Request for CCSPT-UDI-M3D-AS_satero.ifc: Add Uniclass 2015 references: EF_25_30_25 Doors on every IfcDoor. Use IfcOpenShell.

First a look at what the model holds.

```python
import ifcopenshell

model = ifcopenshell.open("CCSPT-UDI-M3D-AS_satero.ifc")
print(model.schema)
print("classifications:", [c.Name for c in model.by_type("IfcClassification")])
for ifc_class in ("IfcDoor", "IfcRoof", "IfcStair", "IfcWall", "IfcWindow"):
    print(ifc_class, len(model.by_type(ifc_class)))
```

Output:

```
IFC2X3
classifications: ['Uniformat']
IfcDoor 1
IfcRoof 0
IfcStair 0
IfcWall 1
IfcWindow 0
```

```python
import ifcopenshell
import ifcopenshell.api.classification

model = ifcopenshell.open("CCSPT-UDI-M3D-AS_satero.ifc")

# IFC2X3 requires Source and Edition and has no link from the project to the system.
system = model.create_entity("IfcClassification", Source="NBS", Edition="2015", Name="Uniclass 2015")

codes = {
    "IfcDoor": ("EF_25_30_25", "Doors"),
}
for ifc_class, (code, name) in codes.items():
    products = model.by_type(ifc_class)
    ifcopenshell.api.classification.add_reference(
        model, products=products, classification=system, identification=code, name=name
    )
    print(code, len(products))

model.write("CCSPT-UDI-M3D-AS_satero_updated.ifc")
```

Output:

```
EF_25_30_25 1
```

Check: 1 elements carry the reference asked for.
